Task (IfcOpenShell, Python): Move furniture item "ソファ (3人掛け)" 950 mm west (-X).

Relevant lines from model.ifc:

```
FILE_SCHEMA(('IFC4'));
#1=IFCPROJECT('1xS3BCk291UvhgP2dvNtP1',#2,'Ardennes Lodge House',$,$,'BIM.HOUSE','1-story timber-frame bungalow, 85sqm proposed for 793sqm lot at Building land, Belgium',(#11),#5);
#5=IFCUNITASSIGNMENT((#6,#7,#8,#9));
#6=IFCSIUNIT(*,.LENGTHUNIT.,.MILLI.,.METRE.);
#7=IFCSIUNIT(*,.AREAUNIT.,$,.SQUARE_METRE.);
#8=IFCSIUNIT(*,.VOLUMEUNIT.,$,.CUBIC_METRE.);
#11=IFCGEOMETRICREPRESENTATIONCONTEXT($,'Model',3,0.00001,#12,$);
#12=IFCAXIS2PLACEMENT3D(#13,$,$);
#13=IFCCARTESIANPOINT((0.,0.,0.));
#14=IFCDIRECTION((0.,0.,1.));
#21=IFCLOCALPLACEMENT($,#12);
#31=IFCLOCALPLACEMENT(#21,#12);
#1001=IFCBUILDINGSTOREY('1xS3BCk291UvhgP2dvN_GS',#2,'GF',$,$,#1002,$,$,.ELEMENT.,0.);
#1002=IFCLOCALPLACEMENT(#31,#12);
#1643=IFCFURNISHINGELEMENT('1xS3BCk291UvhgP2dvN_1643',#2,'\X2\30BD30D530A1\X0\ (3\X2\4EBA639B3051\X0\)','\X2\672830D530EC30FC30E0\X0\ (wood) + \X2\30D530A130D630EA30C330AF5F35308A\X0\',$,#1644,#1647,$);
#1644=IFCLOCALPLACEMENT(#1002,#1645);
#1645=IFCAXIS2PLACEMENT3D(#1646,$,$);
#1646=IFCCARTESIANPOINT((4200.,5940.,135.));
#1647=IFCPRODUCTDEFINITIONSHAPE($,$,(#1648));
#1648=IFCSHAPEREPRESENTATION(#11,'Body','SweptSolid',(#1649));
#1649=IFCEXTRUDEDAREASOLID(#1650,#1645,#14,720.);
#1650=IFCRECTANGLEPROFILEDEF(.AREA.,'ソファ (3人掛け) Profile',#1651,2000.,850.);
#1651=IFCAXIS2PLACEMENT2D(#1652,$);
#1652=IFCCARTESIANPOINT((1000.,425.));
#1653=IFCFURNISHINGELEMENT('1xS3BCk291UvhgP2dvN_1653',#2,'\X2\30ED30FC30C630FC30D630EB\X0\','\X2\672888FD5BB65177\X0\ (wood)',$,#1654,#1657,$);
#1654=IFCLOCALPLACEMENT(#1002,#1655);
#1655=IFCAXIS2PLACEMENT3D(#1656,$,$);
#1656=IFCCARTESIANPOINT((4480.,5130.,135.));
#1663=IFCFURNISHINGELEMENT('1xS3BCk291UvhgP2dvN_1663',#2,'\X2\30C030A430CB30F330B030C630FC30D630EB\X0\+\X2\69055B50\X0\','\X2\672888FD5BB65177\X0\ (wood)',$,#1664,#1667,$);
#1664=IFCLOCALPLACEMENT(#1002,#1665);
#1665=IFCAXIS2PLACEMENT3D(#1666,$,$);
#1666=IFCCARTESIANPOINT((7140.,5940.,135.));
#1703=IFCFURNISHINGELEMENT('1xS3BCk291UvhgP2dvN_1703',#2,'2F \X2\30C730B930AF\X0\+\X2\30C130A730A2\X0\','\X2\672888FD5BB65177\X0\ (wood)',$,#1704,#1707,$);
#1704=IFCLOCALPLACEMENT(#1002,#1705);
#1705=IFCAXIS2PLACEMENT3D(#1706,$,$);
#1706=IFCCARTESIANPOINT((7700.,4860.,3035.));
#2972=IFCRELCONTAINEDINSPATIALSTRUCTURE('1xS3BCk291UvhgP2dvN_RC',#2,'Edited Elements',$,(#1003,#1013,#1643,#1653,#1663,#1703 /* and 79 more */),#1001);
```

```python
import ifcopenshell
import ifcopenshell.api.geometry
import ifcopenshell.util.placement

model = ifcopenshell.open("model.ifc")

item = model.by_guid("1xS3BCk291UvhgP2dvN_1643")
matrix = ifcopenshell.util.placement.get_local_placement(item.ObjectPlacement)
matrix[0, 3] -= 950.0
ifcopenshell.api.geometry.edit_object_placement(model, product=item, matrix=matrix, is_si=False)

print(ifcopenshell.util.placement.get_local_placement(item.ObjectPlacement).round(3) + 0.0)

model.write("model_updated.ifc")
```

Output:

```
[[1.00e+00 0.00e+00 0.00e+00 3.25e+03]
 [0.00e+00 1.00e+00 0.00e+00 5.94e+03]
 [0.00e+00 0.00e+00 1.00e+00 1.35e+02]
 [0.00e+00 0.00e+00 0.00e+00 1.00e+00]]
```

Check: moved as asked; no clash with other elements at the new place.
